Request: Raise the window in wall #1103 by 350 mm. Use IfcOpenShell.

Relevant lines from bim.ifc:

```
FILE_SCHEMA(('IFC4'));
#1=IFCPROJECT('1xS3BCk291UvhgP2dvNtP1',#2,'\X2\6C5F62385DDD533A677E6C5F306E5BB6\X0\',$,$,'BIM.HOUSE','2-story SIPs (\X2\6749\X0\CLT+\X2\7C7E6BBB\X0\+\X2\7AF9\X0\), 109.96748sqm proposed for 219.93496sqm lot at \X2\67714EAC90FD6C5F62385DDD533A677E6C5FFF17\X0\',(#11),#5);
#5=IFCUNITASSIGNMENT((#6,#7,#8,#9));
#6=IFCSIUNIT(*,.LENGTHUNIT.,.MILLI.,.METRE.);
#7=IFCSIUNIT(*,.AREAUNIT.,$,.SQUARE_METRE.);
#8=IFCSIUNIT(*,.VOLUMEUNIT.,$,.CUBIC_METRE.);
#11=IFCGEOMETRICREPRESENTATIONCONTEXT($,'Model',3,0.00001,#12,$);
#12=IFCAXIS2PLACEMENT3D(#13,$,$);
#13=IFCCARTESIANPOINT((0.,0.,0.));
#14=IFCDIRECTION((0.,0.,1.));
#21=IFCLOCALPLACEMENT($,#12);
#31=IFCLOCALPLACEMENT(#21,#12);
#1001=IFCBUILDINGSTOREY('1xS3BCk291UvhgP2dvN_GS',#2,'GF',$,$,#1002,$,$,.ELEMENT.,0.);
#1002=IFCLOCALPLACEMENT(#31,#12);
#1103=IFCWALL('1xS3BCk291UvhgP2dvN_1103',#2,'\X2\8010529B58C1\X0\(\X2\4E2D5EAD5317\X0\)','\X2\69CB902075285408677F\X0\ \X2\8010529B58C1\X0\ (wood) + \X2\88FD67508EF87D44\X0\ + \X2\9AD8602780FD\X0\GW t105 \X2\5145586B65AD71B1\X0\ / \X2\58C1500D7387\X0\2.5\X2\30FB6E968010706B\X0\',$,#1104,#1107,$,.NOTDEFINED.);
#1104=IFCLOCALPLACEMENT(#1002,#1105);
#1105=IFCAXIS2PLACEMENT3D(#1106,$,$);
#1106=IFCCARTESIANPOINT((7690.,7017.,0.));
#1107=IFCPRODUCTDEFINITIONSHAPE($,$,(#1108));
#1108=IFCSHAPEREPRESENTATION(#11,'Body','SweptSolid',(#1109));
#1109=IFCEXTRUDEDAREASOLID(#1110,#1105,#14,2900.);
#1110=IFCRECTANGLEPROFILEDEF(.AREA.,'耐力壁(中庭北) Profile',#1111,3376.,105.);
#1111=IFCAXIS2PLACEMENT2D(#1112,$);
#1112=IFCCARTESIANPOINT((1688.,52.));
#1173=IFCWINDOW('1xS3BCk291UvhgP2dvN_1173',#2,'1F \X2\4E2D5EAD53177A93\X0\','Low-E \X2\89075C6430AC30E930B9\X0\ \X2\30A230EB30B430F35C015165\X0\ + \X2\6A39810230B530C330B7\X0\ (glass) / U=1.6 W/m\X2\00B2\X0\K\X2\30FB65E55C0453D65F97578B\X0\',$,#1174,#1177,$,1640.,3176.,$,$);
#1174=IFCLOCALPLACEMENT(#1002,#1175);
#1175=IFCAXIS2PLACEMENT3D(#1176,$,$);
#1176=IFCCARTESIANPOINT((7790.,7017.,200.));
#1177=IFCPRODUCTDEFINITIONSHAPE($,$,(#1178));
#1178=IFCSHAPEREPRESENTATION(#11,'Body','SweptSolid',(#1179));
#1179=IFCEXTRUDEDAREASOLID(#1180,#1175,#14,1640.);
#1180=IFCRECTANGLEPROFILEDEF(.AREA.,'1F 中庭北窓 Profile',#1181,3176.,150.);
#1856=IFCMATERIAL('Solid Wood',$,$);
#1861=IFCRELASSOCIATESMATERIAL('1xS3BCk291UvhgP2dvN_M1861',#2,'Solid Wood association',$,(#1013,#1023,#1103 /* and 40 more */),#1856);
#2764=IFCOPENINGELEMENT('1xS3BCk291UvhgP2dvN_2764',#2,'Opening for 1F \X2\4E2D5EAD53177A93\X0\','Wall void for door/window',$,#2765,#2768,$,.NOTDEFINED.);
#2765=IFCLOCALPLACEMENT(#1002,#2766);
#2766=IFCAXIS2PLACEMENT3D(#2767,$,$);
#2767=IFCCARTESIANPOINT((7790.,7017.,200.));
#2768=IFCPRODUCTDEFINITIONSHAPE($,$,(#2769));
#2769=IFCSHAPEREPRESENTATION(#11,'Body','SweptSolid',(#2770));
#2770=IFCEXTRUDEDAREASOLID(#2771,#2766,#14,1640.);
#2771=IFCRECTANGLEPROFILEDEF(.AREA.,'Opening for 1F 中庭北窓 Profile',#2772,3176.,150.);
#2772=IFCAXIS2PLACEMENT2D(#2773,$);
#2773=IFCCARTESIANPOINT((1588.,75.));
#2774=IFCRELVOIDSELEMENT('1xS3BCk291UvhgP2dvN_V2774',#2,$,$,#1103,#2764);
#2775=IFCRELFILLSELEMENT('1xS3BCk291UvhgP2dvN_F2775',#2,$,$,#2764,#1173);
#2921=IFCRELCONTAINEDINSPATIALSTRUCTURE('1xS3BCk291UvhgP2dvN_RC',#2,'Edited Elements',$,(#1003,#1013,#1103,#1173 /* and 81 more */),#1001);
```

```python
import numpy as np
import ifcopenshell
import ifcopenshell.api.geometry
import ifcopenshell.util.placement
import ifcopenshell.util.unit

model = ifcopenshell.open("bim.ifc")
unit_scale = ifcopenshell.util.unit.calculate_unit_scale(model)

window = model.by_guid("1xS3BCk291UvhgP2dvN_1173")
opening = window.FillsVoids[0].RelatingOpeningElement
dz = 0.35 / unit_scale

shift = np.array([0.0, 0.0, dz])
# The window is not placed relative to its opening, so move both.
for product in (opening, window):
    matrix = ifcopenshell.util.placement.get_local_placement(product.ObjectPlacement)
    matrix[:3, 3] += shift
    ifcopenshell.api.geometry.edit_object_placement(model, product=product, matrix=matrix, is_si=False)

print(f"moved by {dz * unit_scale:+.3f} m")

model.write("bim-out.ifc")
```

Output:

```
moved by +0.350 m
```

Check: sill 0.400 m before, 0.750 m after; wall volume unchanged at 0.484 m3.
